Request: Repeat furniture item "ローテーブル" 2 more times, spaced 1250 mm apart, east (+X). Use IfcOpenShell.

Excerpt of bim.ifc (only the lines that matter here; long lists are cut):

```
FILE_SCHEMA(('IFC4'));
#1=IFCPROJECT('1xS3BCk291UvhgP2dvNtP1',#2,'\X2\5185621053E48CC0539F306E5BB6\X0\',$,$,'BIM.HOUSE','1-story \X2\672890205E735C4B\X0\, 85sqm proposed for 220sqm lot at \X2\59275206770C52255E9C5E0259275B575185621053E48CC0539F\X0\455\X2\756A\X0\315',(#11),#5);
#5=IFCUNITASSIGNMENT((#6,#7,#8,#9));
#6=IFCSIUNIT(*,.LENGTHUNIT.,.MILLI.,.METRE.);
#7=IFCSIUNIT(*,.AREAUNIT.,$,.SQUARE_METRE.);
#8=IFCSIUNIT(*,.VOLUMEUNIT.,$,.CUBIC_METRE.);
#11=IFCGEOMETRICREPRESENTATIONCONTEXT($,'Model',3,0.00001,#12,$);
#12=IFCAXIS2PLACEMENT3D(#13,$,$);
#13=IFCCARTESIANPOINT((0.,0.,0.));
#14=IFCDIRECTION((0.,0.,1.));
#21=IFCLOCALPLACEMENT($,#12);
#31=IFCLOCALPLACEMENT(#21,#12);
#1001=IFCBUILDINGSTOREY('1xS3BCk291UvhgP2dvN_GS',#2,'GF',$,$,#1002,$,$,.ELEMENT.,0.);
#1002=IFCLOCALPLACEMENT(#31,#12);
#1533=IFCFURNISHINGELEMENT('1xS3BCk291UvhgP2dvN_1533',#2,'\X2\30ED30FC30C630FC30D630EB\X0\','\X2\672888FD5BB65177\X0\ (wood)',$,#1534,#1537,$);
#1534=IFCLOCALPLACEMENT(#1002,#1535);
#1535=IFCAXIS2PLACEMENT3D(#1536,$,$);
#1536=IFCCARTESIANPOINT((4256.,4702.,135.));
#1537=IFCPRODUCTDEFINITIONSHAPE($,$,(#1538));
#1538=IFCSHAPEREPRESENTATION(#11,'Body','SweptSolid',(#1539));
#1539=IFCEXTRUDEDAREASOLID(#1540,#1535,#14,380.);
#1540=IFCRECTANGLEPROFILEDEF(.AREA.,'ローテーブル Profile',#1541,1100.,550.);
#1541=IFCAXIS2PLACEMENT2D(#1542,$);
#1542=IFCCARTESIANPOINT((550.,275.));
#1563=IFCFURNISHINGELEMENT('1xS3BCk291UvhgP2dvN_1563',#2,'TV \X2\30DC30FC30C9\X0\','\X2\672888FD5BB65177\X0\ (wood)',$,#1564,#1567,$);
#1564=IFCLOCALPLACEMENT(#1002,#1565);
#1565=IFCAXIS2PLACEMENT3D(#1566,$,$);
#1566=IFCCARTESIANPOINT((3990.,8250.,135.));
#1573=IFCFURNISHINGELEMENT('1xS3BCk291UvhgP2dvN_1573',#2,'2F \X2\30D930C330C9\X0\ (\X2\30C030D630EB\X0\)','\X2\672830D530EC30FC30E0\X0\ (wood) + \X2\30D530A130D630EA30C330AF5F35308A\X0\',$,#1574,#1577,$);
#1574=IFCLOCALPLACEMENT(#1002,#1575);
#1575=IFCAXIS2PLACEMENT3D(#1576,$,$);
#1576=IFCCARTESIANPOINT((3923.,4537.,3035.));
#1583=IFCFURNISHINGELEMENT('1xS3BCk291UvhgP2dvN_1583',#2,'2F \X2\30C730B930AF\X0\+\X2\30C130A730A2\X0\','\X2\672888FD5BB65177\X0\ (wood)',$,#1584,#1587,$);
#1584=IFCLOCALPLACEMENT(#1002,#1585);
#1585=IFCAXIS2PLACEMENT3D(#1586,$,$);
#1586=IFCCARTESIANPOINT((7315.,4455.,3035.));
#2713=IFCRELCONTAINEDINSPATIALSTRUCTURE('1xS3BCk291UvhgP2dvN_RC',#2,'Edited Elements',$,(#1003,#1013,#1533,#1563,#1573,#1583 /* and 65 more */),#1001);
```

```python
import numpy as np
import ifcopenshell
import ifcopenshell.api.geometry
import ifcopenshell.api.root
import ifcopenshell.util.element
import ifcopenshell.util.placement
import ifcopenshell.util.unit

model = ifcopenshell.open("bim.ifc")
unit_scale = ifcopenshell.util.unit.calculate_unit_scale(model)


def reuse_history(source, copy):
    """copy_class also copies each property set's owner history, people and application; keep the originals."""
    for rel in copy.IsDefinedBy:
        if rel.is_a("IfcRelDefinesByProperties") and (history := rel.RelatingPropertyDefinition.OwnerHistory):
            rel.RelatingPropertyDefinition.OwnerHistory = source.OwnerHistory
            ifcopenshell.util.element.remove_deep2(model, history)


source = model.by_guid("1xS3BCk291UvhgP2dvN_1533")
base = ifcopenshell.util.placement.get_local_placement(source.ObjectPlacement)
step = np.array([1.0, 0.0, 0.0]) * 1.25 / unit_scale

for i in range(1, 3):
    copy = ifcopenshell.api.root.copy_class(model, product=source)
    copy.Representation = ifcopenshell.util.element.copy_deep(
        model, source.Representation, exclude=["IfcGeometricRepresentationContext", "IfcRepresentationMap"]
    )
    reuse_history(source, copy)
    matrix = base.copy()
    matrix[:3, 3] += i * step
    print("added at", matrix[:3, 3].round(3) + 0.0)
    ifcopenshell.api.geometry.edit_object_placement(model, product=copy, matrix=matrix, is_si=False)

model.write("bim_v2.ifc")
```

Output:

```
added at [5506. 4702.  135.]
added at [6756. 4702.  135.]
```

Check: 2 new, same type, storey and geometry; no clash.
